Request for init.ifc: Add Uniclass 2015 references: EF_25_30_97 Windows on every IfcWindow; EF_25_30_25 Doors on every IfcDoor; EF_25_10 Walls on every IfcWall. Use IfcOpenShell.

First a look at what the model holds.

```python
import ifcopenshell

model = ifcopenshell.open("init.ifc")
print(model.schema)
print("classifications:", [c.Name for c in model.by_type("IfcClassification")])
for ifc_class in ("IfcDoor", "IfcRoof", "IfcStair", "IfcWall", "IfcWindow"):
    print(ifc_class, len(model.by_type(ifc_class)))
```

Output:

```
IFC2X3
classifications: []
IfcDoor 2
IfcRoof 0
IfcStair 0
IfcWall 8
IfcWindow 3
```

```python
import ifcopenshell
import ifcopenshell.api.classification

model = ifcopenshell.open("init.ifc")

# IFC2X3 requires Source and Edition and has no link from the project to the system.
system = model.create_entity("IfcClassification", Source="NBS", Edition="2015", Name="Uniclass 2015")

codes = {
    "IfcWindow": ("EF_25_30_97", "Windows"),
    "IfcDoor": ("EF_25_30_25", "Doors"),
    "IfcWall": ("EF_25_10", "Walls"),
}
for ifc_class, (code, name) in codes.items():
    products = model.by_type(ifc_class)
    ifcopenshell.api.classification.add_reference(
        model, products=products, classification=system, identification=code, name=name
    )
    print(code, len(products))

model.write("init-out.ifc")
```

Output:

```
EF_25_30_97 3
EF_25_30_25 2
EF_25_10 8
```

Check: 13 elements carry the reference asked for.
